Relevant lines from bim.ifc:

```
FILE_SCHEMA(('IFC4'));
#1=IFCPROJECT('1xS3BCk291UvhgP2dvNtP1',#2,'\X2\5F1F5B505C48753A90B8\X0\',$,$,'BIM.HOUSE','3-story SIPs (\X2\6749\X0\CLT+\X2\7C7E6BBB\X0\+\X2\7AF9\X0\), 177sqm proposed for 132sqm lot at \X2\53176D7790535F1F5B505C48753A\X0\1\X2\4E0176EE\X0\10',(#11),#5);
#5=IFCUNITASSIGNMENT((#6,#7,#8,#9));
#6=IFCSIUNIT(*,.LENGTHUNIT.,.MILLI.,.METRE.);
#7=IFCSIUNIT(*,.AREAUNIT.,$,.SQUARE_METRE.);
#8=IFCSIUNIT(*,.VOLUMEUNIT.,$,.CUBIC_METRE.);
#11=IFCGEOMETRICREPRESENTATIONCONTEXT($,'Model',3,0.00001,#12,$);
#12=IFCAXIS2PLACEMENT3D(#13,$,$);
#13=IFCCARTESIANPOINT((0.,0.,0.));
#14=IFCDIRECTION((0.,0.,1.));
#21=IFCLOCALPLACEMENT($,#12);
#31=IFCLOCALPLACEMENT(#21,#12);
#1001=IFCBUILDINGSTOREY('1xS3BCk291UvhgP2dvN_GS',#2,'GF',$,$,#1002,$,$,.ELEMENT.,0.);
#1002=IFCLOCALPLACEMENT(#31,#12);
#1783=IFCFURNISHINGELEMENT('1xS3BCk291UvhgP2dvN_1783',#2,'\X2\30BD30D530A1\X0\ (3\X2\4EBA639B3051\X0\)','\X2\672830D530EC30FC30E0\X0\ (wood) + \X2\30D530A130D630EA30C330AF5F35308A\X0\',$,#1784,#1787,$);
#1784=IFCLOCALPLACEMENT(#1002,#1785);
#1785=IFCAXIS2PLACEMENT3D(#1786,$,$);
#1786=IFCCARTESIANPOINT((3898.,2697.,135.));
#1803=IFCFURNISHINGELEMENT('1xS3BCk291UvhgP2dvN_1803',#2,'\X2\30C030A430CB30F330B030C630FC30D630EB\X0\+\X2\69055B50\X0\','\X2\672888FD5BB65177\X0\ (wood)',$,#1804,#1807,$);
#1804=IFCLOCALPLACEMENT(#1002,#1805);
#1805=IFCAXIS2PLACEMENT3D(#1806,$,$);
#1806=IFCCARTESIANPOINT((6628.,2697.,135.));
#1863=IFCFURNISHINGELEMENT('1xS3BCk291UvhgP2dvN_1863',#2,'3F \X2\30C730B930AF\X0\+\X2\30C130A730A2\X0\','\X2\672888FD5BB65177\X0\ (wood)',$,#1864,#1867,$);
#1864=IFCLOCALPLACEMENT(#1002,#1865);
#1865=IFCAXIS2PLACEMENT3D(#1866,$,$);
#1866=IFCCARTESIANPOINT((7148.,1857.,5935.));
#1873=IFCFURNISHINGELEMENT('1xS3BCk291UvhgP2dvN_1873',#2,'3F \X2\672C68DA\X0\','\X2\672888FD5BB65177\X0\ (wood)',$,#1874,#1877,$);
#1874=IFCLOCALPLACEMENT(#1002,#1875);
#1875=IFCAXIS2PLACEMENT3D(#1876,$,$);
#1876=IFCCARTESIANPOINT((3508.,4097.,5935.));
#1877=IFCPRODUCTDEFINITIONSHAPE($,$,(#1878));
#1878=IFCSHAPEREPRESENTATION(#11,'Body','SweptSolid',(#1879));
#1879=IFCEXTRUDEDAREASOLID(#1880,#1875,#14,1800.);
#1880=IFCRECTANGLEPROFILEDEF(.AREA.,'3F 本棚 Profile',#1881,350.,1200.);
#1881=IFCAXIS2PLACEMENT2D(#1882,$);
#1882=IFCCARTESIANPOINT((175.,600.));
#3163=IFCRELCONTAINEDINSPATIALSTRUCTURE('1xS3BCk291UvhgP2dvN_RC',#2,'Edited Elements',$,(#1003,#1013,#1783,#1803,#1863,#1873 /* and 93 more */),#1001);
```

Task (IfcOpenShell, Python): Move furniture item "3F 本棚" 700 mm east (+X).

```python
import ifcopenshell
import ifcopenshell.api.geometry
import ifcopenshell.util.placement
import ifcopenshell.util.unit

model = ifcopenshell.open("bim.ifc")
unit_scale = ifcopenshell.util.unit.calculate_unit_scale(model)

item = model.by_guid("1xS3BCk291UvhgP2dvN_1873")
matrix = ifcopenshell.util.placement.get_local_placement(item.ObjectPlacement)
matrix[0, 3] += 0.7 / unit_scale
ifcopenshell.api.geometry.edit_object_placement(model, product=item, matrix=matrix, is_si=False)

print(ifcopenshell.util.placement.get_local_placement(item.ObjectPlacement).round(3) + 0.0)

model.write("bim-out.ifc")
```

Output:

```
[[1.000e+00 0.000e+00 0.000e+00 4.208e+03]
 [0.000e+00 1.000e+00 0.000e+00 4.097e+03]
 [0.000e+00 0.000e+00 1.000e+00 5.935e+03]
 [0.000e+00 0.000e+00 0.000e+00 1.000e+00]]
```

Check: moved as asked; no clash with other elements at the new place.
